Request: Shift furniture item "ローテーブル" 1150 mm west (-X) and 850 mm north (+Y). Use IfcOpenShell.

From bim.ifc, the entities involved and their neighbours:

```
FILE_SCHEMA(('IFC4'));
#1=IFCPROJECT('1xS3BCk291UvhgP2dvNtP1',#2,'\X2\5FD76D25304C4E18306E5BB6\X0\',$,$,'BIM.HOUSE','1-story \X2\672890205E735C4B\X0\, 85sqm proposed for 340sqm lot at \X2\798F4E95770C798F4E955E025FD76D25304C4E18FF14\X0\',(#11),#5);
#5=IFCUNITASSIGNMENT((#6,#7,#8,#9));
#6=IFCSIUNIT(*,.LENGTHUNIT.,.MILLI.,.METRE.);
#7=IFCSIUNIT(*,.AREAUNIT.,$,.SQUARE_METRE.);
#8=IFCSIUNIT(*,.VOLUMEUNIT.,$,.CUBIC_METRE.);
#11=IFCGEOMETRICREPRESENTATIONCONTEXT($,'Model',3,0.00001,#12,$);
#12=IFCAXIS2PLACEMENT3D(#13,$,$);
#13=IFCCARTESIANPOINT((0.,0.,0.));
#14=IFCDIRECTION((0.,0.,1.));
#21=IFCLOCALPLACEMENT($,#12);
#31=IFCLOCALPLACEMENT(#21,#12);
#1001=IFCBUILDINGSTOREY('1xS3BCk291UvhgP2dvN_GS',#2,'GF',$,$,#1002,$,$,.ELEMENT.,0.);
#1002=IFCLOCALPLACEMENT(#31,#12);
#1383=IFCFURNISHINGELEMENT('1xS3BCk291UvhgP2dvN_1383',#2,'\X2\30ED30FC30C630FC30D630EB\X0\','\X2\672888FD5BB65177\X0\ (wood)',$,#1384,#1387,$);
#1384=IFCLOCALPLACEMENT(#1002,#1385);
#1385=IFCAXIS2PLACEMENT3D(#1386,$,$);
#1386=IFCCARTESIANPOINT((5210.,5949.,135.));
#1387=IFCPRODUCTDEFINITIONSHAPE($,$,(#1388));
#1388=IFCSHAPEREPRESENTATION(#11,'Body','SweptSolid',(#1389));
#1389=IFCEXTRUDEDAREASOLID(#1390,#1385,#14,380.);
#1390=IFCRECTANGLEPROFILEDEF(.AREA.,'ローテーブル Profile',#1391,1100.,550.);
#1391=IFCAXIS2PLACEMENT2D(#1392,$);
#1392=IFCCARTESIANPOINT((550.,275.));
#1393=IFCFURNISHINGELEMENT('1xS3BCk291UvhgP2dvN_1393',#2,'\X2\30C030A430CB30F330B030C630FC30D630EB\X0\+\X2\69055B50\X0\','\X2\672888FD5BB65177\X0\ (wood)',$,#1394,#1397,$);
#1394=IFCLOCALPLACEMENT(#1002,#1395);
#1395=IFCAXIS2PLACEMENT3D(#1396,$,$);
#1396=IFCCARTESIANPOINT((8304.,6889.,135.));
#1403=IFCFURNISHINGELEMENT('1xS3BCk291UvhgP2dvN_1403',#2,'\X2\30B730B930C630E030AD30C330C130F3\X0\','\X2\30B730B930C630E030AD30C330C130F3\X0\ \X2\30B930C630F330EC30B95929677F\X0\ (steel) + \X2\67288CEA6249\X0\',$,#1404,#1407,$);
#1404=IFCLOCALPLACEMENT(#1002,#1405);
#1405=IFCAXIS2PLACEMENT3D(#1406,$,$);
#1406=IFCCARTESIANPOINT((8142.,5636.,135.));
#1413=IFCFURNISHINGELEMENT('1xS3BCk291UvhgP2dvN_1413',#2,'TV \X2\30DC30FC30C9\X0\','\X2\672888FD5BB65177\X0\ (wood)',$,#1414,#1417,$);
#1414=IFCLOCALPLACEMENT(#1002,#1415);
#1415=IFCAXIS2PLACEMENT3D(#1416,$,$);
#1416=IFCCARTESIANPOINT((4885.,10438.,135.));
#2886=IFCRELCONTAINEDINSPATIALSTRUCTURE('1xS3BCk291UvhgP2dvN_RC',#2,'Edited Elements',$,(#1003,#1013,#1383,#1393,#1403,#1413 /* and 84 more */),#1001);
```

```python
import ifcopenshell
import ifcopenshell.api.geometry
import ifcopenshell.util.placement

model = ifcopenshell.open("bim.ifc")

item = model.by_guid("1xS3BCk291UvhgP2dvN_1383")
matrix = ifcopenshell.util.placement.get_local_placement(item.ObjectPlacement)
matrix[0, 3] -= 1150.0
matrix[1, 3] += 850.0
ifcopenshell.api.geometry.edit_object_placement(model, product=item, matrix=matrix, is_si=False)

print(ifcopenshell.util.placement.get_local_placement(item.ObjectPlacement).round(3) + 0.0)

model.write("bim-out.ifc")
```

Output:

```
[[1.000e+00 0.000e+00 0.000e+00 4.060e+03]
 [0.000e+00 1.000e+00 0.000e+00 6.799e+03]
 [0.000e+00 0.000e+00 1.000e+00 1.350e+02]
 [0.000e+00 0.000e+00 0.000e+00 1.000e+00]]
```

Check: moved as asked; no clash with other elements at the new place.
